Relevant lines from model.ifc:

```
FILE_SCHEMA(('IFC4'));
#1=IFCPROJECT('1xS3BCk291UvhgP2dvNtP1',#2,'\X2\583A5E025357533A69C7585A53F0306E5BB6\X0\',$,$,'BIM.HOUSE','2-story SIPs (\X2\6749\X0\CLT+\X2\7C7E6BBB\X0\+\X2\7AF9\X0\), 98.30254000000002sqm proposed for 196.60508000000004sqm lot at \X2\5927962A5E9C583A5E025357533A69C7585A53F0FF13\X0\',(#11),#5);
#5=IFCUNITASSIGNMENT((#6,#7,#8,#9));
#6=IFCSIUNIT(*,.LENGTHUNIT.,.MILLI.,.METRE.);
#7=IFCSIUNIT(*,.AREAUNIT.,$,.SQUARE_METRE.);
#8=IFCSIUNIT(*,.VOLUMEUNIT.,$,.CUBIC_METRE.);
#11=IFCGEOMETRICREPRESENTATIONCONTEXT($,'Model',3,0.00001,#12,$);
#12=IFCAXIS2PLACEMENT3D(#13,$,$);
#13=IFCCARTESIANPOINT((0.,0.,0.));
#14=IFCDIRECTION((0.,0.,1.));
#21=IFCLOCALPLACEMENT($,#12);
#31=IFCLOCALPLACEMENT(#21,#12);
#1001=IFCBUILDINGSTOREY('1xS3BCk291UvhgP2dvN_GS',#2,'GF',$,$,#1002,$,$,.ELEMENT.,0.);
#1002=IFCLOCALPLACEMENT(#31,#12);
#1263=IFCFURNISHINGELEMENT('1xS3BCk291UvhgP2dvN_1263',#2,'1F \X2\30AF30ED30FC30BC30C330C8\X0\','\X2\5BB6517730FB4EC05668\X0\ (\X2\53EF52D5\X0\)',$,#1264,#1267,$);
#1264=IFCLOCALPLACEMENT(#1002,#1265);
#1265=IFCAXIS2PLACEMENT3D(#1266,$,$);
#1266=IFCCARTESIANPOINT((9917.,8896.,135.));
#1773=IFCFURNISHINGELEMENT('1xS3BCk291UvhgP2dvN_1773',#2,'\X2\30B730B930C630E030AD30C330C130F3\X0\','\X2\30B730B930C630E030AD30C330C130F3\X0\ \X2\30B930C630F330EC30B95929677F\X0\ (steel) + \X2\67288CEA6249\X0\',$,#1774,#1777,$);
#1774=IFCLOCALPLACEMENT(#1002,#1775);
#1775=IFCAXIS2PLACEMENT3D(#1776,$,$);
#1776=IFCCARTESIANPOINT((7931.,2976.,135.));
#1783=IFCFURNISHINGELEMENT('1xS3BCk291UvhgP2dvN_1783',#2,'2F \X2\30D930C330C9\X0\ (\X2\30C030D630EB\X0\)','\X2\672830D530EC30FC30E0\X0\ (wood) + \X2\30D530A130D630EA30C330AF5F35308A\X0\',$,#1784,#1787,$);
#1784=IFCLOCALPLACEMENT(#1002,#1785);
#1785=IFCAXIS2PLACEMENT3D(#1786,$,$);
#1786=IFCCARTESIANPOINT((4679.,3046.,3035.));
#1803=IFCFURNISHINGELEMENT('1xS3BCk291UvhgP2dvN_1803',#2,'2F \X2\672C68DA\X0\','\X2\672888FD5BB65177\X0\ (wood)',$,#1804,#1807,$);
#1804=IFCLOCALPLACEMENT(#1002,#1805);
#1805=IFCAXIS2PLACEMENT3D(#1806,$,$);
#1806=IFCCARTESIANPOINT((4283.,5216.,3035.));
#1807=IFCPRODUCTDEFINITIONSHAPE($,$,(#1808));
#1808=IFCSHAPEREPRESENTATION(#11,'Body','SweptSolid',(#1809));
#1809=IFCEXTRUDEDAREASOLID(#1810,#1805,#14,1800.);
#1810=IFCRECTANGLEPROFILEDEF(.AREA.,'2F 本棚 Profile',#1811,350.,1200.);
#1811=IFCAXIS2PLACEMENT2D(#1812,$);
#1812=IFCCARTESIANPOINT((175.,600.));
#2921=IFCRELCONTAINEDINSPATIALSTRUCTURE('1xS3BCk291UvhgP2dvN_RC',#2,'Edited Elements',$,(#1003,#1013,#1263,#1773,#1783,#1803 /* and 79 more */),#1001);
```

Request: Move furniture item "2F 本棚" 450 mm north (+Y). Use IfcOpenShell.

```python
import ifcopenshell
import ifcopenshell.api.geometry
import ifcopenshell.util.placement

model = ifcopenshell.open("model.ifc")

item = model.by_guid("1xS3BCk291UvhgP2dvN_1803")
matrix = ifcopenshell.util.placement.get_local_placement(item.ObjectPlacement)
matrix[1, 3] += 450.0
ifcopenshell.api.geometry.edit_object_placement(model, product=item, matrix=matrix, is_si=False)

print(ifcopenshell.util.placement.get_local_placement(item.ObjectPlacement).round(3) + 0.0)

model.write("model_rev.ifc")
```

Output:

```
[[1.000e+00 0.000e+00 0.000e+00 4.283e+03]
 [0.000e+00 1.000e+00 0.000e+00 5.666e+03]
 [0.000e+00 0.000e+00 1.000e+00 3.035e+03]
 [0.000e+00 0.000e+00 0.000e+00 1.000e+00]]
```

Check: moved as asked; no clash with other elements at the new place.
